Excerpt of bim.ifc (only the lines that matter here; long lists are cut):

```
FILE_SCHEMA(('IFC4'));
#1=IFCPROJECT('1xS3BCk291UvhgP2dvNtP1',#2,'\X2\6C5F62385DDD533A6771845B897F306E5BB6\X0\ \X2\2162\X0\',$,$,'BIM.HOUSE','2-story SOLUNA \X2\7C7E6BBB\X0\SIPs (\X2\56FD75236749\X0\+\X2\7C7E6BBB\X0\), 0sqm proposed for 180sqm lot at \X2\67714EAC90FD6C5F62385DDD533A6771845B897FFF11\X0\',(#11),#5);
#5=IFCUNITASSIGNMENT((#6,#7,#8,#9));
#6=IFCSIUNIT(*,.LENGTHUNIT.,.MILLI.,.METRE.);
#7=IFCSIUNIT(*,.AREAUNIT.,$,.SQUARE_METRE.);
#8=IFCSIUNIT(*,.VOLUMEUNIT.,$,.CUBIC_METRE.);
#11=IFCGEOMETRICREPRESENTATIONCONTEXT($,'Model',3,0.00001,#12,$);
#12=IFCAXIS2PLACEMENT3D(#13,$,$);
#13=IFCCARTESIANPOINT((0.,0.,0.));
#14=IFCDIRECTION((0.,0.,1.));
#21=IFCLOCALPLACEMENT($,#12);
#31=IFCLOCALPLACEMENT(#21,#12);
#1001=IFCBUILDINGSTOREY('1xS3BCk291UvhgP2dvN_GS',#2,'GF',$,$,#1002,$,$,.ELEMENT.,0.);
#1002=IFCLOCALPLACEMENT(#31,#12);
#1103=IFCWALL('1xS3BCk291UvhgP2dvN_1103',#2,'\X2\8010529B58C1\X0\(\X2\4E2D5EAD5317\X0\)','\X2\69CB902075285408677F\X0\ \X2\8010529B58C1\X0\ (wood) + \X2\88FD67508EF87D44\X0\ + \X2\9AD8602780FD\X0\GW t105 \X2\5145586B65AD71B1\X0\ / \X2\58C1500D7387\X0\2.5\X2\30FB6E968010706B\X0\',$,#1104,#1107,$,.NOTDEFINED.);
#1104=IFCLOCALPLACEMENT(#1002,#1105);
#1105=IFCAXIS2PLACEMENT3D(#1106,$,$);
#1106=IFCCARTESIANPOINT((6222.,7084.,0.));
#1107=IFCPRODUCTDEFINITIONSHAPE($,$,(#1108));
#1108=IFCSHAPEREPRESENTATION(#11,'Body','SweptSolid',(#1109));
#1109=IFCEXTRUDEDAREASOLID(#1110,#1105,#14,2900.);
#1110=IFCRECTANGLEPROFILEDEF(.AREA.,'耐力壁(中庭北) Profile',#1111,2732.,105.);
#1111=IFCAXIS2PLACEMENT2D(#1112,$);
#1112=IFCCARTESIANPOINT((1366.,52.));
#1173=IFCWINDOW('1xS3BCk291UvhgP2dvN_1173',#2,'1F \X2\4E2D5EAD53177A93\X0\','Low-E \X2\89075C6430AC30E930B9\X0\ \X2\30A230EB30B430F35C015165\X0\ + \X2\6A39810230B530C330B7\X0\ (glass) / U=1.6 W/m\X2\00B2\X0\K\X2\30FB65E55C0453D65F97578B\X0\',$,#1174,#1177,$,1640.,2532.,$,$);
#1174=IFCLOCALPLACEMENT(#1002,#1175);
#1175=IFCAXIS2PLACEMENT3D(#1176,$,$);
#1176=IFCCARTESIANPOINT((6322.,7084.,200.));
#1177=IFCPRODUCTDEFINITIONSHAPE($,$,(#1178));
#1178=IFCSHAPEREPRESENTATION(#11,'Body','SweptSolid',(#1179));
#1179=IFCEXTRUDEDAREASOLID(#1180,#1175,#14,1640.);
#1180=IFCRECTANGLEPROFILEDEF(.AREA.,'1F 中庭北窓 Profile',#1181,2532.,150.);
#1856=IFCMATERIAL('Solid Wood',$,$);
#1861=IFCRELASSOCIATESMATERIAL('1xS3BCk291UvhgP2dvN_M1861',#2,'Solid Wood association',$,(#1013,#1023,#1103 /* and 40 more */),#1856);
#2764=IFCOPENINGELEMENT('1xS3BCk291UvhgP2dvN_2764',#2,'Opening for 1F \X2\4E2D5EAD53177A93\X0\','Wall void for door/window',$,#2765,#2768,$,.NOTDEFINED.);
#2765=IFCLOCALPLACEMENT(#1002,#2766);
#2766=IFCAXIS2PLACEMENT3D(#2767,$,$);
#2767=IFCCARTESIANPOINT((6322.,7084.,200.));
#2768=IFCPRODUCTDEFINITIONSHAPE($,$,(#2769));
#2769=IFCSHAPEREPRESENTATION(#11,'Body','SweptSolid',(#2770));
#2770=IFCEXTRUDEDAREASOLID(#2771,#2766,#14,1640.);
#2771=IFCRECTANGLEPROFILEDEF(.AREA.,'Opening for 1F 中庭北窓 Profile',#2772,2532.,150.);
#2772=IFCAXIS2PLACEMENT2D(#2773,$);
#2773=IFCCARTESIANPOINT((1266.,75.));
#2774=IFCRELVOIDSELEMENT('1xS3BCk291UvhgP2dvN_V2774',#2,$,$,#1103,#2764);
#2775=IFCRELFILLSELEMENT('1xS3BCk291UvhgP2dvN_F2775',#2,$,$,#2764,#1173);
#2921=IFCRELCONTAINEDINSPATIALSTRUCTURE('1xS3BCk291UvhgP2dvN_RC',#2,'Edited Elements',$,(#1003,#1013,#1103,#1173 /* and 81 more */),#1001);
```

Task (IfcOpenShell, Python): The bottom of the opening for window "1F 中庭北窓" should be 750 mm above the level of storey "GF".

```python
import numpy as np
import ifcopenshell
import ifcopenshell.api.geometry
import ifcopenshell.geom
import ifcopenshell.util.element
import ifcopenshell.util.placement
import ifcopenshell.util.shape
import ifcopenshell.util.unit

model = ifcopenshell.open("bim.ifc")
unit_scale = ifcopenshell.util.unit.calculate_unit_scale(model)

window = model.by_guid("1xS3BCk291UvhgP2dvN_1173")
opening = window.FillsVoids[0].RelatingOpeningElement
storey = ifcopenshell.util.element.get_container(window, ifc_class="IfcBuildingStorey")
level = ifcopenshell.util.placement.get_local_placement(storey.ObjectPlacement)[2, 3]

# The opening's origin need not be at the sill, so measure its lowest point.
shape = ifcopenshell.geom.create_shape(ifcopenshell.geom.settings(), opening)
bottom = ifcopenshell.util.shape.get_shape_bottom_elevation(shape, shape.geometry) / unit_scale
dz = level + 750.0 - bottom

shift = np.array([0.0, 0.0, dz])
# The window is not placed relative to its opening, so move both.
for product in (opening, window):
    matrix = ifcopenshell.util.placement.get_local_placement(product.ObjectPlacement)
    matrix[:3, 3] += shift
    ifcopenshell.api.geometry.edit_object_placement(model, product=product, matrix=matrix, is_si=False)

print(f"moved by {dz * unit_scale:+.3f} m")

model.write("bim_edited.ifc")
```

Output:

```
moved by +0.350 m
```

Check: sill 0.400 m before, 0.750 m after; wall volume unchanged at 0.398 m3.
